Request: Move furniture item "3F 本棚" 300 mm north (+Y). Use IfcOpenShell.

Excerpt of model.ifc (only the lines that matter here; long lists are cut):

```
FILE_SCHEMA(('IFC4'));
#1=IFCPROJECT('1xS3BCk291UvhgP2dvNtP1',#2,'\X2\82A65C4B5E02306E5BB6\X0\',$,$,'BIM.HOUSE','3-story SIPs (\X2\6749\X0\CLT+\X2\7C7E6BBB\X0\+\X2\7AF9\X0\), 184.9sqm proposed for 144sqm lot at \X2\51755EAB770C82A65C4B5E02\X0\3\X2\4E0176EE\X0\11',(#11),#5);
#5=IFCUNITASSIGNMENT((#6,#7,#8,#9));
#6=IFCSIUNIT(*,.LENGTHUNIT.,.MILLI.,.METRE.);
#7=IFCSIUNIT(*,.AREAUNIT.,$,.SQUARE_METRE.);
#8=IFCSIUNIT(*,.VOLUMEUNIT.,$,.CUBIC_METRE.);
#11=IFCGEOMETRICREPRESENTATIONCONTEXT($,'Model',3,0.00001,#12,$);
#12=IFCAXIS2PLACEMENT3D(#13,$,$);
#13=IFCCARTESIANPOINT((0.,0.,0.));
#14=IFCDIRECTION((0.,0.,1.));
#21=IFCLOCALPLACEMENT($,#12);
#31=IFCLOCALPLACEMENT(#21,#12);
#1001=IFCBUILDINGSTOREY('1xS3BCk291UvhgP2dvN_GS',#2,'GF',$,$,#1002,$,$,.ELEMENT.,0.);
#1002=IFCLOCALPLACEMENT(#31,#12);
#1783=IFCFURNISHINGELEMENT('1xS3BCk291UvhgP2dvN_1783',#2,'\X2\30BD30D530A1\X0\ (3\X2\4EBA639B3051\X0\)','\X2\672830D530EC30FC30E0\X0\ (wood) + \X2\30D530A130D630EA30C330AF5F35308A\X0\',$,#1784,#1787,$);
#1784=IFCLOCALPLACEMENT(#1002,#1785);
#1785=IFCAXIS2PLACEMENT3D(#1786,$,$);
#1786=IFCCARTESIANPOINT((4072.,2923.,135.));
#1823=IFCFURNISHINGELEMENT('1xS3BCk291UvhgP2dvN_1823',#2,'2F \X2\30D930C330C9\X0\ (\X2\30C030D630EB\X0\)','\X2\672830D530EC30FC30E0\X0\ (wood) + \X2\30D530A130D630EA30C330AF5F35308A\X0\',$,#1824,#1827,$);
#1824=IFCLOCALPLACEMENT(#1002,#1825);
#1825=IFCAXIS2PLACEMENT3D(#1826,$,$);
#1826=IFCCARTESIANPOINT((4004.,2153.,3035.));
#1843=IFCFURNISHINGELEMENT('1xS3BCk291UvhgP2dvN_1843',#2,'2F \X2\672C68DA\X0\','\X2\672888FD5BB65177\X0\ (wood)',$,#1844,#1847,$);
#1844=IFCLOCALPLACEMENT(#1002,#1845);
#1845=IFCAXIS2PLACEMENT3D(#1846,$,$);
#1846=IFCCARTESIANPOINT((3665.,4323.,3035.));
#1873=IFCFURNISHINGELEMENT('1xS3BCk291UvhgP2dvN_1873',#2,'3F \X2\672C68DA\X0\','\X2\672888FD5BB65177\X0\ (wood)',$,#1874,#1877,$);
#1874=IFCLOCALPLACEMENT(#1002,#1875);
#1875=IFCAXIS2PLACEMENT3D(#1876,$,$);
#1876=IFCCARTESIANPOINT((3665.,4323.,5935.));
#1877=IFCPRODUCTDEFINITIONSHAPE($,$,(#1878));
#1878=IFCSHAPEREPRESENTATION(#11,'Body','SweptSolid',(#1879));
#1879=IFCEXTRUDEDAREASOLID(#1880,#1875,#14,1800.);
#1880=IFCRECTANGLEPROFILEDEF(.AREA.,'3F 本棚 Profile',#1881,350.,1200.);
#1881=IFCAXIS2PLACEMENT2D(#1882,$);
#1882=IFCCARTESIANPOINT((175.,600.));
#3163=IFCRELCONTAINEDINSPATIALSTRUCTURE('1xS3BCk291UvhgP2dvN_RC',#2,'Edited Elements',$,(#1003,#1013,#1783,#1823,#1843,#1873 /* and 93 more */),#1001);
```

```python
import ifcopenshell
import ifcopenshell.api.geometry
import ifcopenshell.util.placement
import ifcopenshell.util.unit

model = ifcopenshell.open("model.ifc")
unit_scale = ifcopenshell.util.unit.calculate_unit_scale(model)

item = model.by_id(1873)
matrix = ifcopenshell.util.placement.get_local_placement(item.ObjectPlacement)
matrix[1, 3] += 0.3 / unit_scale
ifcopenshell.api.geometry.edit_object_placement(model, product=item, matrix=matrix, is_si=False)

print(ifcopenshell.util.placement.get_local_placement(item.ObjectPlacement).round(3) + 0.0)

model.write("model_updated.ifc")
```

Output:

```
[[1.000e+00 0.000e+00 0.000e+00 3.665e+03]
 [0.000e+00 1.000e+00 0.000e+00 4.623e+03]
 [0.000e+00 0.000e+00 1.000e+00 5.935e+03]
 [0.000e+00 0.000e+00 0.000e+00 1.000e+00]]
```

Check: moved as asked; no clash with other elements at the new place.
